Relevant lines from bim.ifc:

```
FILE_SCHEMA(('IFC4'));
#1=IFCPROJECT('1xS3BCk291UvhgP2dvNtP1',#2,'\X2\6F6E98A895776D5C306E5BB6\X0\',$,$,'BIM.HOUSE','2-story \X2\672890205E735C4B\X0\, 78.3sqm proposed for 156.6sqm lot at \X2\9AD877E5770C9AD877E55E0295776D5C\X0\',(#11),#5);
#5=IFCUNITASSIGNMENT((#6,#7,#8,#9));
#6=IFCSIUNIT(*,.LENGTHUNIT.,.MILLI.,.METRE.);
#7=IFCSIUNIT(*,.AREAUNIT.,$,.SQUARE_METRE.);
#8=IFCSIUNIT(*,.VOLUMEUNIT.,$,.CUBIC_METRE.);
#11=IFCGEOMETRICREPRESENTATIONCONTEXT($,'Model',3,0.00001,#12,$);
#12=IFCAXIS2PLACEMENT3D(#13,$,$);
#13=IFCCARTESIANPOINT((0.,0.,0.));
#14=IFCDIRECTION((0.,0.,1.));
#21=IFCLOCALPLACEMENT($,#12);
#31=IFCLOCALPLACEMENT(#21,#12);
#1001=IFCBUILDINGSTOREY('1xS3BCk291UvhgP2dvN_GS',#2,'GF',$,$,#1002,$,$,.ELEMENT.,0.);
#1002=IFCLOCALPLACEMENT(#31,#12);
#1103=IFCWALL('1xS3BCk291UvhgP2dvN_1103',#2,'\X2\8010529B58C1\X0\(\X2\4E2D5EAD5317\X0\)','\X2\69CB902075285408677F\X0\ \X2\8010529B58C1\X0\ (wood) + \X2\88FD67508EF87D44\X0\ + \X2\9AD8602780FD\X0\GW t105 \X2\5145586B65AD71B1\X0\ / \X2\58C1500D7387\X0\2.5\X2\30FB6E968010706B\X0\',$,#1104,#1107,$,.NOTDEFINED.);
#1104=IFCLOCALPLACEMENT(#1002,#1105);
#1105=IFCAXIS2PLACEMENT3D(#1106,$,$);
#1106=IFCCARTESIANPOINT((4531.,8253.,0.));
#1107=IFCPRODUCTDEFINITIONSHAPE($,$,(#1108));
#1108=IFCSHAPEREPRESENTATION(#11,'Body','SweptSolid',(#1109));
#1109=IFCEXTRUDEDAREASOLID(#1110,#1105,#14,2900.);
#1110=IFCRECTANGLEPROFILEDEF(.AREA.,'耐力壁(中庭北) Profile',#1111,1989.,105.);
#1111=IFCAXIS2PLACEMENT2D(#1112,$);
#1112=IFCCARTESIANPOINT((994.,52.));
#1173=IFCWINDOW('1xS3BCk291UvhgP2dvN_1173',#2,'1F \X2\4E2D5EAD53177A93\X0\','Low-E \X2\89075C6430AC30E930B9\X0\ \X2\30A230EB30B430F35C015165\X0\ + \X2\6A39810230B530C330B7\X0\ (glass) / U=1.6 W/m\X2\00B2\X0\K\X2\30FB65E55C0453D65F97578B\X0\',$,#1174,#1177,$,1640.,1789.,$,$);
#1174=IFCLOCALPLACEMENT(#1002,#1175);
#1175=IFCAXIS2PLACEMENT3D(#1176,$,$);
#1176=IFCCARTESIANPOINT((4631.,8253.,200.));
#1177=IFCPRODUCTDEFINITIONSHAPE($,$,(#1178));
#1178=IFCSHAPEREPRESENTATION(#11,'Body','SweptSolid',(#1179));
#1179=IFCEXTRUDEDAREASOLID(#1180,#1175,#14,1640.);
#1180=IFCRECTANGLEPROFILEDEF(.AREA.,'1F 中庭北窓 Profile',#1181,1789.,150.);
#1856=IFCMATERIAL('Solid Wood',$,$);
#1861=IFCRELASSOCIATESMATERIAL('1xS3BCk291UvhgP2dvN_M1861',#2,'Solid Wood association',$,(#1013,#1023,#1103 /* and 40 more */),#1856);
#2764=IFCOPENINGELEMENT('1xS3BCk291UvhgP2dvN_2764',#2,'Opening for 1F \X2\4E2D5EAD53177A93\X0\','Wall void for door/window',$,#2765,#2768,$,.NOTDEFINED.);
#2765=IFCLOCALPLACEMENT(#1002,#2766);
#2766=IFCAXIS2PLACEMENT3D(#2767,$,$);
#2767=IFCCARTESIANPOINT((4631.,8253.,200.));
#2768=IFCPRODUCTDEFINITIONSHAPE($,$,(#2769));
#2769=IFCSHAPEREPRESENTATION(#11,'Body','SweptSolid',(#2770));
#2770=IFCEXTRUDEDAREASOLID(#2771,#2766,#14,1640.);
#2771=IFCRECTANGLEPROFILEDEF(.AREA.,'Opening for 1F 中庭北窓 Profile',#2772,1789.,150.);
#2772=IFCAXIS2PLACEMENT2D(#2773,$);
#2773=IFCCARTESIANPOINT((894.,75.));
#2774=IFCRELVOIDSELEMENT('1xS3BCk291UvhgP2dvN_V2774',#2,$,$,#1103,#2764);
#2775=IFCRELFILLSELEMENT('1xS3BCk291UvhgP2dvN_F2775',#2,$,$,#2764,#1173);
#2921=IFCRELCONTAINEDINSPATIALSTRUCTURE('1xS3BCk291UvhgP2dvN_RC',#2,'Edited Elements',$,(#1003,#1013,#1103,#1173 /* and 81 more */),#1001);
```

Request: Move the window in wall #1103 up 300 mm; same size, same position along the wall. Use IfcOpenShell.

```python
import numpy as np
import ifcopenshell
import ifcopenshell.api.geometry
import ifcopenshell.util.placement
import ifcopenshell.util.unit

model = ifcopenshell.open("bim.ifc")
unit_scale = ifcopenshell.util.unit.calculate_unit_scale(model)

window = model.by_guid("1xS3BCk291UvhgP2dvN_1173")
opening = window.FillsVoids[0].RelatingOpeningElement
dz = 0.3 / unit_scale

shift = np.array([0.0, 0.0, dz])
# The window is not placed relative to its opening, so move both.
for product in (opening, window):
    matrix = ifcopenshell.util.placement.get_local_placement(product.ObjectPlacement)
    matrix[:3, 3] += shift
    ifcopenshell.api.geometry.edit_object_placement(model, product=product, matrix=matrix, is_si=False)

print(f"moved by {dz * unit_scale:+.3f} m")

model.write("bim_updated.ifc")
```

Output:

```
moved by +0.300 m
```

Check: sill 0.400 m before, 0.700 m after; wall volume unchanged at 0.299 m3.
